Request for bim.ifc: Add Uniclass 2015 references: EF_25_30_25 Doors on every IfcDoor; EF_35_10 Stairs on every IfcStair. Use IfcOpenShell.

First a look at what the model holds.

```python
import ifcopenshell

model = ifcopenshell.open("bim.ifc")
print(model.schema)
print("classifications:", [c.Name for c in model.by_type("IfcClassification")])
for ifc_class in ("IfcDoor", "IfcRoof", "IfcStair", "IfcWall", "IfcWindow"):
    print(ifc_class, len(model.by_type(ifc_class)))
```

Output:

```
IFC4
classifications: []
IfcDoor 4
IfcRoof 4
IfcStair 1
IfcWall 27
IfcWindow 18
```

```python
import ifcopenshell
import ifcopenshell.api.classification

model = ifcopenshell.open("bim.ifc")

system = ifcopenshell.api.classification.add_classification(model, classification="Uniclass 2015")

codes = {
    "IfcDoor": ("EF_25_30_25", "Doors"),
    "IfcStair": ("EF_35_10", "Stairs"),
}
for ifc_class, (code, name) in codes.items():
    products = model.by_type(ifc_class)
    ifcopenshell.api.classification.add_reference(
        model, products=products, classification=system, identification=code, name=name
    )
    print(code, len(products))

model.write("bim-out.ifc")
```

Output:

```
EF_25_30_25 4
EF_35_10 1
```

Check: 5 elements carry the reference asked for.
